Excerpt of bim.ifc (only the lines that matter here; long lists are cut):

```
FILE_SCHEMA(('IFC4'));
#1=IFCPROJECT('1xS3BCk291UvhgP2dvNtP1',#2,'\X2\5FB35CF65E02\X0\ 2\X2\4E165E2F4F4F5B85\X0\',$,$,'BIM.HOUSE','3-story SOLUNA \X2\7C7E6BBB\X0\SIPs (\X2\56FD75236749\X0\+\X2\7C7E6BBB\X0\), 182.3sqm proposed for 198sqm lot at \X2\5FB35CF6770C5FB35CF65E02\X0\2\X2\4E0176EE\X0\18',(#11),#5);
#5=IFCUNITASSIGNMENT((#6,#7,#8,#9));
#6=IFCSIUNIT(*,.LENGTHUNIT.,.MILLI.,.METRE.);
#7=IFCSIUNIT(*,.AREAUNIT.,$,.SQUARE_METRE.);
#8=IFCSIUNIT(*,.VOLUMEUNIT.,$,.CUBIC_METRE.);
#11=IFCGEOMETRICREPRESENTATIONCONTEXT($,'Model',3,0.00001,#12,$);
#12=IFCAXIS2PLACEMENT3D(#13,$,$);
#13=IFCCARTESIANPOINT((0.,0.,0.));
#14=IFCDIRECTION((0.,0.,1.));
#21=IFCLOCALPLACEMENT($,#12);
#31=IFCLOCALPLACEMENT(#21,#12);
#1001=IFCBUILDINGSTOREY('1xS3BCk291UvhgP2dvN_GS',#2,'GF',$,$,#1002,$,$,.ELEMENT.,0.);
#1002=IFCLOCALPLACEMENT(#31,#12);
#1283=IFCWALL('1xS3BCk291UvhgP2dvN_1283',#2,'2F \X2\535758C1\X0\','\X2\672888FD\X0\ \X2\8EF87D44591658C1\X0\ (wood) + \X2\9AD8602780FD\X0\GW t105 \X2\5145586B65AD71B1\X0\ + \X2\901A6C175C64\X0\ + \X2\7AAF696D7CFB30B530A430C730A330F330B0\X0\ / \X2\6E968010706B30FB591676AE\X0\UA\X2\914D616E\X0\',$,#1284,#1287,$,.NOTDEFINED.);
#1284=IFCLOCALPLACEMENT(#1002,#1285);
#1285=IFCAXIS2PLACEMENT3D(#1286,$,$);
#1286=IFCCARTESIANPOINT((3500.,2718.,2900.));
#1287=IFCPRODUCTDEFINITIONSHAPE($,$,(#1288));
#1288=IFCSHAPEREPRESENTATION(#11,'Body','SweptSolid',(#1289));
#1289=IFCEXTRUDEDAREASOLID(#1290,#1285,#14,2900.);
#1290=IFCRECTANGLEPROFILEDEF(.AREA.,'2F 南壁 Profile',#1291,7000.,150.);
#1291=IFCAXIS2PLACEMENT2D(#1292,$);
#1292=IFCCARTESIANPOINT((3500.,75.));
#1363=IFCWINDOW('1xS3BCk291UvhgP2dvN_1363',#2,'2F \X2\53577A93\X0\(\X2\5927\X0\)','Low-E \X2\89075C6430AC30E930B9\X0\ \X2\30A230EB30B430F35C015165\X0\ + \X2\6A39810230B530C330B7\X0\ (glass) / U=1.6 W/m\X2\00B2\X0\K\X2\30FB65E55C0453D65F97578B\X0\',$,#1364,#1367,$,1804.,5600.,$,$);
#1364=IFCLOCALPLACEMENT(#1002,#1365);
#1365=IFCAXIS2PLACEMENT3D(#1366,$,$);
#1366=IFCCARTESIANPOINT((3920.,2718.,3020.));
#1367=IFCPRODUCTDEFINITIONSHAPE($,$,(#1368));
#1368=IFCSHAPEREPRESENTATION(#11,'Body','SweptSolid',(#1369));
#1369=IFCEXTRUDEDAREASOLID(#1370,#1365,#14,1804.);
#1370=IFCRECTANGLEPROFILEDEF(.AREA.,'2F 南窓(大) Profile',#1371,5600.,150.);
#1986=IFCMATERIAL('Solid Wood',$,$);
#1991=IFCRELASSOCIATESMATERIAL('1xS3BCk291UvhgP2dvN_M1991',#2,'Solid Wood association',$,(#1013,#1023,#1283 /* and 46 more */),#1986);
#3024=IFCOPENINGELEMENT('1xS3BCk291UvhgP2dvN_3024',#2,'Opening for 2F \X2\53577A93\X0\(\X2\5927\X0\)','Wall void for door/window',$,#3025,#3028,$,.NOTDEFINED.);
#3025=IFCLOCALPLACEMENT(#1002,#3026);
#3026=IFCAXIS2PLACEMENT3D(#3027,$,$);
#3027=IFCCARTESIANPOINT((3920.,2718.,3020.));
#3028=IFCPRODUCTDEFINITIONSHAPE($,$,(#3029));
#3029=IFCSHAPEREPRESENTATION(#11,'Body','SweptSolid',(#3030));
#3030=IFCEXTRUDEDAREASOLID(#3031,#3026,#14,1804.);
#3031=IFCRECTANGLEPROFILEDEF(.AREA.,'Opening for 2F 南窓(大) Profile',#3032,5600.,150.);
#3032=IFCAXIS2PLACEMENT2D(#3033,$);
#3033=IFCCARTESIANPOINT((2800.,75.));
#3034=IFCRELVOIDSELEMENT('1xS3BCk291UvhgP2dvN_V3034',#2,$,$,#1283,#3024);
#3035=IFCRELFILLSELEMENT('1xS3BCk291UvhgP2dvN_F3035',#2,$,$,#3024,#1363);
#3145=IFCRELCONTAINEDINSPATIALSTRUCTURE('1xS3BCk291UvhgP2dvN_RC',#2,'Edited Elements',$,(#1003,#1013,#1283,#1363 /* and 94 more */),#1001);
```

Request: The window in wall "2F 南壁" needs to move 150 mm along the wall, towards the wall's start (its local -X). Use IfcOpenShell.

```python
import ifcopenshell
import ifcopenshell.api.geometry
import ifcopenshell.util.placement
import ifcopenshell.util.unit

model = ifcopenshell.open("bim.ifc")
unit_scale = ifcopenshell.util.unit.calculate_unit_scale(model)

window = model.by_id(1363)
opening = window.FillsVoids[0].RelatingOpeningElement
wall = opening.VoidsElements[0].RelatingBuildingElement

wall_matrix = ifcopenshell.util.placement.get_local_placement(wall.ObjectPlacement)
shift = wall_matrix[:3, 0] * -0.15 / unit_scale
before = ifcopenshell.util.placement.get_local_placement(window.ObjectPlacement)[:3, 3].copy()

# The window is not placed relative to its opening, so move both.
for product in (opening, window):
    matrix = ifcopenshell.util.placement.get_local_placement(product.ObjectPlacement)
    matrix[:3, 3] += shift
    ifcopenshell.api.geometry.edit_object_placement(model, product=product, matrix=matrix, is_si=False)

after = ifcopenshell.util.placement.get_local_placement(window.ObjectPlacement)[:3, 3]
print("window moved by", (after - before).round(3) + 0.0)

model.write("bim_rev.ifc")
```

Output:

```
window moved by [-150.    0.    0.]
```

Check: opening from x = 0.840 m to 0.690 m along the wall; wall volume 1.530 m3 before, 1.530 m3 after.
